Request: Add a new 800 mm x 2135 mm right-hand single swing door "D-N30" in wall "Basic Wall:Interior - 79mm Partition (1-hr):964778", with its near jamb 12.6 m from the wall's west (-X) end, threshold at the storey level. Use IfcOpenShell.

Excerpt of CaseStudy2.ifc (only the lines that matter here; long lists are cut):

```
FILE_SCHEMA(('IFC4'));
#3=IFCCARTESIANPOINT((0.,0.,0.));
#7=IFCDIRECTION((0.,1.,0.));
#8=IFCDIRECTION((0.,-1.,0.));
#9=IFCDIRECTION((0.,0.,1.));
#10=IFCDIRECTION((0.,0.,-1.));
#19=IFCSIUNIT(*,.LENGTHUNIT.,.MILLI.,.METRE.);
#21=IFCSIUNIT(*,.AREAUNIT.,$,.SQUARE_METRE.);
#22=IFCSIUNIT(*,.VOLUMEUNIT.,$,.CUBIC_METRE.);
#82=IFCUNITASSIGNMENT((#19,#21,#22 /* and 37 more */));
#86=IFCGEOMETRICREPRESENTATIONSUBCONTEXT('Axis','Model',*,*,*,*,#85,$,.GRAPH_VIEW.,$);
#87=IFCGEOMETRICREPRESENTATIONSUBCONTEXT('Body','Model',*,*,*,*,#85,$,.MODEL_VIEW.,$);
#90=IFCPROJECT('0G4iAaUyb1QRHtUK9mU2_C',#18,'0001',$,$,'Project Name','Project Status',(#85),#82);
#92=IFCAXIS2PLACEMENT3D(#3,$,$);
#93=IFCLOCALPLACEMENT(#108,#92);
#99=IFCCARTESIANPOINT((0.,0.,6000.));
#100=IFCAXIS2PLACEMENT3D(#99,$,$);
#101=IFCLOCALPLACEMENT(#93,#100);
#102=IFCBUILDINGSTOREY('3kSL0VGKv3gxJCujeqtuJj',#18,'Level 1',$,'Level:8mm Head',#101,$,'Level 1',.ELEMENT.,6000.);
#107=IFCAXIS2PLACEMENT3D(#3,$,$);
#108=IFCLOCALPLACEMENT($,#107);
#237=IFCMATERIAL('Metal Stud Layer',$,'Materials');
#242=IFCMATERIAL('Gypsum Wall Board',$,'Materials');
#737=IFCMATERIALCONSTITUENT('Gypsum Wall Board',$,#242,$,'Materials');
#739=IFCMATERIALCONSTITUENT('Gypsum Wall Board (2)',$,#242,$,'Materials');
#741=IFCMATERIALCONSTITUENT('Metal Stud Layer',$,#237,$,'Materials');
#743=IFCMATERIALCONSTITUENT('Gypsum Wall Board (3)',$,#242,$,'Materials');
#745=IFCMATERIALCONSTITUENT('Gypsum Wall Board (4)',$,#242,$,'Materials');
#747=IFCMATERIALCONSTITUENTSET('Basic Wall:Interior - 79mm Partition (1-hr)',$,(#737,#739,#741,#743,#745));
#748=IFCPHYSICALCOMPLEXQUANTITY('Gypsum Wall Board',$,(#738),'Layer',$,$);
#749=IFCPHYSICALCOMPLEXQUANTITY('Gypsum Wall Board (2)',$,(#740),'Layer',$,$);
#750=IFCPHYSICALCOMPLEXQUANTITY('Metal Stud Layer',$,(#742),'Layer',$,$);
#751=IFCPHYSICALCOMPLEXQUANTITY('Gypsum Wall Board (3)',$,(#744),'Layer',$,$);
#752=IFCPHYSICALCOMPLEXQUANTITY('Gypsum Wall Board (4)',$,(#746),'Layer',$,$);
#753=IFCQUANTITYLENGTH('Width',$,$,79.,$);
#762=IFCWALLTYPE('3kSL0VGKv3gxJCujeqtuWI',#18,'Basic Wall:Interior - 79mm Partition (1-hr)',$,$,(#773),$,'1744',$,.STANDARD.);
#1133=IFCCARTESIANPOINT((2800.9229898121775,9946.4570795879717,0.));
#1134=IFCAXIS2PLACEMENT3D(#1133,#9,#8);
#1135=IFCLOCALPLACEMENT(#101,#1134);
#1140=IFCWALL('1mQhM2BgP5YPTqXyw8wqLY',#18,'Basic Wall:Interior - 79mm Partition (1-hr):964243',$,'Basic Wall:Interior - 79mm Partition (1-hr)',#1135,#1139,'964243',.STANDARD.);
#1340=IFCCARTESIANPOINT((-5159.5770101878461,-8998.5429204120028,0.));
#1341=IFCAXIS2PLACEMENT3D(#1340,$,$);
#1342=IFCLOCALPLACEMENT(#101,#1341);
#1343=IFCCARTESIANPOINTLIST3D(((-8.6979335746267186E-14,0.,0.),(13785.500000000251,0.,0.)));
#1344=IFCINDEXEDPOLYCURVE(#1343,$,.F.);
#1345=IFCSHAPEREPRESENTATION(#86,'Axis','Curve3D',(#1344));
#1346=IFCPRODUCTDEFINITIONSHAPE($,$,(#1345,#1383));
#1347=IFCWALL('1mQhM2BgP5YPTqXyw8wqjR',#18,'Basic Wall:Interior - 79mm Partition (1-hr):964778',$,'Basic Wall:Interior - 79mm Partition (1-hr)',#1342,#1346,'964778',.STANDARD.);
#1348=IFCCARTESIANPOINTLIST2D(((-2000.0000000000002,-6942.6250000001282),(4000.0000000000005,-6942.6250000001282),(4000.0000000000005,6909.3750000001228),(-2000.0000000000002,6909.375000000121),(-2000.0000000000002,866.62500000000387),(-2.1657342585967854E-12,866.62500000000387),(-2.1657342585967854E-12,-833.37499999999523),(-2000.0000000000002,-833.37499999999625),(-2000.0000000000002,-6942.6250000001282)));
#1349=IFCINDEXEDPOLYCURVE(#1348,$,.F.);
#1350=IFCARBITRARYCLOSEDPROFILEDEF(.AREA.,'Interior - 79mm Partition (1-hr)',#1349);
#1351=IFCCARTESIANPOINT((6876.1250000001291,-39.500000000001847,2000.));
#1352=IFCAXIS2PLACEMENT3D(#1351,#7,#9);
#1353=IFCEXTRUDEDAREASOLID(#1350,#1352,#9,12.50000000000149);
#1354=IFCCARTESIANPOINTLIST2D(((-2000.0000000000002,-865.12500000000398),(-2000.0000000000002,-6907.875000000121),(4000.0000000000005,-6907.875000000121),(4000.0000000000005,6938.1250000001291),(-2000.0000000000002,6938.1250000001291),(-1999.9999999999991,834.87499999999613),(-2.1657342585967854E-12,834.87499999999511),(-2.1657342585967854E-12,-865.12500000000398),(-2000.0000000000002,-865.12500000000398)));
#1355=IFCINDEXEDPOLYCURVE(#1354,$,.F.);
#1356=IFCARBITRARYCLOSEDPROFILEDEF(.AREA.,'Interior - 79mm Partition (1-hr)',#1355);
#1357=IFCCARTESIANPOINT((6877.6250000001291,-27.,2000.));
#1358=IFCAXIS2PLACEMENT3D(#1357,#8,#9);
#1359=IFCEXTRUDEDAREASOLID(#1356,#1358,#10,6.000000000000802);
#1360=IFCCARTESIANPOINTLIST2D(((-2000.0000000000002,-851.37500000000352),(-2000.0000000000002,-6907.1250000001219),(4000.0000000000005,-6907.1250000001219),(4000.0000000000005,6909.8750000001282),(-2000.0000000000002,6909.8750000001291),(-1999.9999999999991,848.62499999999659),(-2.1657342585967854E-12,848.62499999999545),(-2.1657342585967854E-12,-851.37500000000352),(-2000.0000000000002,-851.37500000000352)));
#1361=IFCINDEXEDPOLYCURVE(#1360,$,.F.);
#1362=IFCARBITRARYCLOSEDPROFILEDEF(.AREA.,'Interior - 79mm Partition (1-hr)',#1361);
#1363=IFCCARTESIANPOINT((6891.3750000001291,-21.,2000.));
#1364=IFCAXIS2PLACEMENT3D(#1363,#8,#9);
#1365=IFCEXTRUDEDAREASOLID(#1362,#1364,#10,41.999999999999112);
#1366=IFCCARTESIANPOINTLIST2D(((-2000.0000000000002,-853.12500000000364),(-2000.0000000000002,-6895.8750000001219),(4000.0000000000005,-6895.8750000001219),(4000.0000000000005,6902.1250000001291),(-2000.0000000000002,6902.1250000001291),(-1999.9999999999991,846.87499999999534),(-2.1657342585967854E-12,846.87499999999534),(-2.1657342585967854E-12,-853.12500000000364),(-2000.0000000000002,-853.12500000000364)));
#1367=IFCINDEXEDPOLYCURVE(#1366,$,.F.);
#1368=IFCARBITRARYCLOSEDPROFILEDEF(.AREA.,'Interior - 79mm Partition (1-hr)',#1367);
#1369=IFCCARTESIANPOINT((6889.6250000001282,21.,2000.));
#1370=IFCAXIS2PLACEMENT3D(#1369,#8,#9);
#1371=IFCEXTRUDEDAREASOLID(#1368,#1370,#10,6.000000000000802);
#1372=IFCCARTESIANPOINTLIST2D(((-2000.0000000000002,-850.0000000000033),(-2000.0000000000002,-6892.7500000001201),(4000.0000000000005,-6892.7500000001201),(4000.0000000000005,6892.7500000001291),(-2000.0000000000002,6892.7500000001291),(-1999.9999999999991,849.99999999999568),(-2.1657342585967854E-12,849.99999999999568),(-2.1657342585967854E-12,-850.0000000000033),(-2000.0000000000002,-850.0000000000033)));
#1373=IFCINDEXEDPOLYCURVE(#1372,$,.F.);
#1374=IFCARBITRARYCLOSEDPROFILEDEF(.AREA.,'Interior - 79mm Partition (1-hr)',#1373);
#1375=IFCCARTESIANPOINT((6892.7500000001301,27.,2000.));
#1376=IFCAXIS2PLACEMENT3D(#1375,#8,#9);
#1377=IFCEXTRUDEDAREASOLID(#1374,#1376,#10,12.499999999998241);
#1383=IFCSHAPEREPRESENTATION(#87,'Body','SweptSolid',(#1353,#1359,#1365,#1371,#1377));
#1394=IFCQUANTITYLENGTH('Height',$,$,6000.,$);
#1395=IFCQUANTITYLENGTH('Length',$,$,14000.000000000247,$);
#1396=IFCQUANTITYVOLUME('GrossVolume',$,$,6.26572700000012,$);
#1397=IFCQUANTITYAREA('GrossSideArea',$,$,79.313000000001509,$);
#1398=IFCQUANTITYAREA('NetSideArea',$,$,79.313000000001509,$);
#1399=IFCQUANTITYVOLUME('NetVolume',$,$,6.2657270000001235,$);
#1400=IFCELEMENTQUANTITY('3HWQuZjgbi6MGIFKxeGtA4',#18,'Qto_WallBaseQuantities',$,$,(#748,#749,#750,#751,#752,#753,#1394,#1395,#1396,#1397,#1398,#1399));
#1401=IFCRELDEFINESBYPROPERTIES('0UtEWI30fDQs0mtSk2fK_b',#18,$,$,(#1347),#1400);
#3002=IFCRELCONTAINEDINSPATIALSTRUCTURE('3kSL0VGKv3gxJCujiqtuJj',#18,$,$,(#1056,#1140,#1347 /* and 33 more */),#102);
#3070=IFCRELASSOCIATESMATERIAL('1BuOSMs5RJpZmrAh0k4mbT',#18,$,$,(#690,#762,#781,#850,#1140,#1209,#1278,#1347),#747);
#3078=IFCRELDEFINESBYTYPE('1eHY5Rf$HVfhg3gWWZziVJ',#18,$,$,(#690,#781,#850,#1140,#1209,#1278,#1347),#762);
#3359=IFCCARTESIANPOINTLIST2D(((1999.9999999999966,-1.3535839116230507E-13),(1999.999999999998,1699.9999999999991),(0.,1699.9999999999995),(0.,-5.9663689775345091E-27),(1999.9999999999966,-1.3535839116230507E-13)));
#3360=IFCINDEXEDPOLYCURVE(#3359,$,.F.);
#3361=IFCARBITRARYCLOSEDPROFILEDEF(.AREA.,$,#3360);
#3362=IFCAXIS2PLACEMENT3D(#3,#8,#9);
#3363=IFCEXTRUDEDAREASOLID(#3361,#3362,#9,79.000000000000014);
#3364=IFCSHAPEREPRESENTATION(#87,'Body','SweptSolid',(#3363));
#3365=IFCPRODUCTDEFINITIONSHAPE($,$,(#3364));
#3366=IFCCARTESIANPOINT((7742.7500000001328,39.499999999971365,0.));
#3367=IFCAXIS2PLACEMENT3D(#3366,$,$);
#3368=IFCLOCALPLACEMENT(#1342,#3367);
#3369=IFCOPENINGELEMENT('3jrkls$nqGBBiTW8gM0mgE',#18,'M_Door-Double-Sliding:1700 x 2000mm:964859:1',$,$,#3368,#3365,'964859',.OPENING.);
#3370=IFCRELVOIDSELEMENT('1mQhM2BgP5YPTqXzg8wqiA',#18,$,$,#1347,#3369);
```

```python
import numpy as np
import ifcopenshell
import ifcopenshell.api.feature
import ifcopenshell.api.geometry
import ifcopenshell.api.pset
import ifcopenshell.api.root
import ifcopenshell.api.spatial
import ifcopenshell.geom
import ifcopenshell.util.element
import ifcopenshell.util.placement
import ifcopenshell.util.representation
import ifcopenshell.util.shape
import ifcopenshell.util.unit

model = ifcopenshell.open("CaseStudy2.ifc")
unit_scale = ifcopenshell.util.unit.calculate_unit_scale(model)
area_scale = ifcopenshell.util.unit.calculate_unit_scale(model, "AREAUNIT")
volume_scale = ifcopenshell.util.unit.calculate_unit_scale(model, "VOLUMEUNIT")
settings = ifcopenshell.geom.settings()


def volume(element):
    """Net volume in cubic metres, openings subtracted."""
    shape = ifcopenshell.geom.create_shape(settings, element)
    return ifcopenshell.util.shape.get_volume(shape.geometry)


wall = model.by_guid("1mQhM2BgP5YPTqXyw8wqjR")
storey = ifcopenshell.util.element.get_container(wall, ifc_class="IfcBuildingStorey")
context = ifcopenshell.util.representation.get_context(model, "Model", "Body", "MODEL_VIEW")
before = volume(wall)

width, height, from_end, sill = 0.8, 2.135, 12.6, 0.0  # metres

# The wall runs along its own X axis, and the end named is its -X end.
wall_shape = ifcopenshell.geom.create_shape(settings, wall)
x, y, z = ifcopenshell.util.shape.get_vertices(wall_shape.geometry).T
start = x.min() + from_end
face, thickness = float(y.min()), float(y.max() - y.min())
wall_matrix = ifcopenshell.util.placement.get_local_placement(wall.ObjectPlacement)
level = ifcopenshell.util.placement.get_local_placement(storey.ObjectPlacement)[2, 3]


def in_wall(x, y):
    """Placement at x, y metres in the wall's axes, at sill height."""
    matrix = wall_matrix.copy()
    matrix[:, 3] = wall_matrix @ np.array([x / unit_scale, y / unit_scale, 0.0, 1.0])
    matrix[2, 3] = level + sill / unit_scale
    return matrix


# Opening: a box that overshoots both wall faces by 50 mm.
opening = ifcopenshell.api.root.create_entity(model, ifc_class="IfcOpeningElement", predefined_type="OPENING")
box = ifcopenshell.api.geometry.add_wall_representation(
    model, context=context, length=width, height=height, thickness=thickness + 0.1
)
ifcopenshell.api.geometry.assign_representation(model, product=opening, representation=box)
ifcopenshell.api.geometry.edit_object_placement(model, product=opening, matrix=in_wall(start, face - 0.05), is_si=False)
ifcopenshell.api.feature.add_feature(model, feature=opening, element=wall)

door = ifcopenshell.api.root.create_entity(model, ifc_class="IfcDoor", name="D-N30", predefined_type="DOOR")
door.OverallWidth, door.OverallHeight = width / unit_scale, height / unit_scale
door.OperationType = "SINGLE_SWING_RIGHT"
body = ifcopenshell.api.geometry.add_door_representation(
    model,
    context=context,
    overall_width=door.OverallWidth,
    overall_height=door.OverallHeight,
    operation_type="SINGLE_SWING_RIGHT",
    lining_properties={"LiningDepth": thickness / unit_scale, "ThresholdDepth": thickness / unit_scale},
)
ifcopenshell.api.geometry.assign_representation(model, product=door, representation=body)
ifcopenshell.api.spatial.assign_container(model, products=[door], relating_structure=storey)
ifcopenshell.api.feature.add_filling(model, opening=opening, element=door)

# The lining spans the wall, so the door starts at the wall face.
ifcopenshell.api.geometry.edit_object_placement(model, product=door, matrix=in_wall(start, face), is_si=False)

after = volume(wall)

# Update the wall's stored quantities.
qto = model.by_id(ifcopenshell.util.element.get_pset(wall, "Qto_WallBaseQuantities", should_inherit=False)["id"])
ifcopenshell.api.pset.edit_qto(model, qto=qto, properties={
    "NetSideArea": after / thickness / area_scale,
    "NetVolume": after / volume_scale,
})

print(f"wall volume {before:.3f} -> {after:.3f} m3")

model.write("CaseStudy2_v2.ifc")
```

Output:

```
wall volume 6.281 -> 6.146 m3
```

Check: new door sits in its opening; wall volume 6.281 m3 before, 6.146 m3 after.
